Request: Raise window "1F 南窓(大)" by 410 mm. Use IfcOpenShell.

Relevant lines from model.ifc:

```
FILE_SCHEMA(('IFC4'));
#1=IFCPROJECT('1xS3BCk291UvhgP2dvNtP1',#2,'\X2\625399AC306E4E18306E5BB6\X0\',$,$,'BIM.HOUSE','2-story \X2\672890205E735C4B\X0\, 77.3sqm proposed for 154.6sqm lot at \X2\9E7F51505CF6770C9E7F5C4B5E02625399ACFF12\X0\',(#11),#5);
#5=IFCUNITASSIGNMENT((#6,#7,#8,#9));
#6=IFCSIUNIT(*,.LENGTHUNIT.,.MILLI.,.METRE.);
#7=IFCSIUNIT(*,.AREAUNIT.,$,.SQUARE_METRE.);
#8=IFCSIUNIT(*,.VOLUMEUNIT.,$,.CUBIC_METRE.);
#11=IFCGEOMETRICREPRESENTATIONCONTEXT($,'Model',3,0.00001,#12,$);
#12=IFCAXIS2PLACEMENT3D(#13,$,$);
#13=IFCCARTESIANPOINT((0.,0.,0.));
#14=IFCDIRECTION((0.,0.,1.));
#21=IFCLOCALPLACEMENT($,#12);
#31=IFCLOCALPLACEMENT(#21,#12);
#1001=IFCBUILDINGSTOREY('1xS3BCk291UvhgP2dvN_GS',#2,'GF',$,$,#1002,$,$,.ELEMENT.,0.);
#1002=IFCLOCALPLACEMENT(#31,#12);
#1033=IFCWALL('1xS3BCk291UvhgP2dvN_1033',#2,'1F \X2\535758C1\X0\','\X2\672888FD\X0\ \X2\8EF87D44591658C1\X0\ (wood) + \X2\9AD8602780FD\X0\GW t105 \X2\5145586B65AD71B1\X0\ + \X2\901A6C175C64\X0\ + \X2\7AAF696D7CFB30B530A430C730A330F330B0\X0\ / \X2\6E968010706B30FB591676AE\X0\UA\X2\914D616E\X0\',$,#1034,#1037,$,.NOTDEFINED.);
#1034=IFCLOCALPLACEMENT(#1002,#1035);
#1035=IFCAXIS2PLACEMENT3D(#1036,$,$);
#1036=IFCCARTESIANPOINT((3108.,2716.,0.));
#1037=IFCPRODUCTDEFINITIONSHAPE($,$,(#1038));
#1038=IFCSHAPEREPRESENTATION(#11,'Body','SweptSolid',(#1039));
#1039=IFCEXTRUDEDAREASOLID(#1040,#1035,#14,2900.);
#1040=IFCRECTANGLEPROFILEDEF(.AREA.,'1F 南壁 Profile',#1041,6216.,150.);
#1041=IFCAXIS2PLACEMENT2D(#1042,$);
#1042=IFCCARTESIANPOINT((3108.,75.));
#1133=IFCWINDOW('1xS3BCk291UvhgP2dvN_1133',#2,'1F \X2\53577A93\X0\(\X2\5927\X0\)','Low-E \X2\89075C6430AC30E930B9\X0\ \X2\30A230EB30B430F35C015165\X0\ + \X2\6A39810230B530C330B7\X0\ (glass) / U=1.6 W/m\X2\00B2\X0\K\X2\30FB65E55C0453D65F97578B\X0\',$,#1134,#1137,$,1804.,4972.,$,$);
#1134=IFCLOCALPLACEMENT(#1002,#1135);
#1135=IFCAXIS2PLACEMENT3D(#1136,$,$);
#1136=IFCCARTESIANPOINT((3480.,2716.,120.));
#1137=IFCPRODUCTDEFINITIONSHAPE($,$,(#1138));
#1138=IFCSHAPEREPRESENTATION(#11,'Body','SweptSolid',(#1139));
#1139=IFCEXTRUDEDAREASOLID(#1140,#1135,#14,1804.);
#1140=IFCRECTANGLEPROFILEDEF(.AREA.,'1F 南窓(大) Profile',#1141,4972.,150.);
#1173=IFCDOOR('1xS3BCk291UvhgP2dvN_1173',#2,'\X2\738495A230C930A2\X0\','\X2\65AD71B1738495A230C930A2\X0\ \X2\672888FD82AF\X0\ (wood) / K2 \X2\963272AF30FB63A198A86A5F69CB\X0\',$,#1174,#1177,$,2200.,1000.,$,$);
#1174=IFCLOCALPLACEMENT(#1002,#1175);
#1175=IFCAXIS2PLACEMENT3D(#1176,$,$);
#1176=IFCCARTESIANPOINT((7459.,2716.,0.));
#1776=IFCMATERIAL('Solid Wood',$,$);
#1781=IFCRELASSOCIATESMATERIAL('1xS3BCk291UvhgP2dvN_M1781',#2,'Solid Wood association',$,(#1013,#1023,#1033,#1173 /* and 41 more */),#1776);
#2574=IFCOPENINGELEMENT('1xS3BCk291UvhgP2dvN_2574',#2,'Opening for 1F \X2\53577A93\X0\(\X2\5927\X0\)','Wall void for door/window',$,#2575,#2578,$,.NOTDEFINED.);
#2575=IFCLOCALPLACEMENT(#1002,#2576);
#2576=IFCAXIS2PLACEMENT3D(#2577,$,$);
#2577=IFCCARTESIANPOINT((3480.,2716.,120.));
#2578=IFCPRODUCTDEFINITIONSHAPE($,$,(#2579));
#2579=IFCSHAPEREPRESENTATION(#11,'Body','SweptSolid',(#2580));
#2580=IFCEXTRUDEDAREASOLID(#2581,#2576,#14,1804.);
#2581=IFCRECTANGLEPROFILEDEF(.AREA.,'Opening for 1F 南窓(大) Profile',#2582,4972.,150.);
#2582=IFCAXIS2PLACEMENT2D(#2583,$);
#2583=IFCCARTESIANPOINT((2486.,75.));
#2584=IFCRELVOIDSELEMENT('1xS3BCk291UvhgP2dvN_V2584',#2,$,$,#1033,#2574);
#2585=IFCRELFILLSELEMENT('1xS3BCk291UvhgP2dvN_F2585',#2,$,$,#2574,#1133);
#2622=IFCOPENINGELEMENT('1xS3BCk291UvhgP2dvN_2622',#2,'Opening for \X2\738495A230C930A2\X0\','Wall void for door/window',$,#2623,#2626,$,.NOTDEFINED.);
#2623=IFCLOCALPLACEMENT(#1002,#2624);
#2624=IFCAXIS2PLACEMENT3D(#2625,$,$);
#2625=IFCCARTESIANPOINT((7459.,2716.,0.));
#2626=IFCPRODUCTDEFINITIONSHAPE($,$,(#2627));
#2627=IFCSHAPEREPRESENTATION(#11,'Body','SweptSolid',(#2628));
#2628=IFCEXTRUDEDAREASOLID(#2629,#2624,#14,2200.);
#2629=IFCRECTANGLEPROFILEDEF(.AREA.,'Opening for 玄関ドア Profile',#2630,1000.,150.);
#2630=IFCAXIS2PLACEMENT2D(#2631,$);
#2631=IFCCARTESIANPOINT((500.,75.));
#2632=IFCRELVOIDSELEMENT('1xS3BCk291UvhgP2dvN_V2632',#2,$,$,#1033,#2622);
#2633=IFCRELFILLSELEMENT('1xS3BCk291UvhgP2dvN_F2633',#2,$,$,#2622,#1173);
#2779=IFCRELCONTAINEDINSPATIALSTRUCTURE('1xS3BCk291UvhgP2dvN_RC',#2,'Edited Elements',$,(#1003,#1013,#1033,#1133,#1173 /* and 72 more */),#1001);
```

```python
import numpy as np
import ifcopenshell
import ifcopenshell.api.geometry
import ifcopenshell.util.placement
import ifcopenshell.util.unit

model = ifcopenshell.open("model.ifc")
unit_scale = ifcopenshell.util.unit.calculate_unit_scale(model)

window = model.by_id(1133)
opening = window.FillsVoids[0].RelatingOpeningElement
dz = 0.41 / unit_scale

shift = np.array([0.0, 0.0, dz])
# The window is not placed relative to its opening, so move both.
for product in (opening, window):
    matrix = ifcopenshell.util.placement.get_local_placement(product.ObjectPlacement)
    matrix[:3, 3] += shift
    ifcopenshell.api.geometry.edit_object_placement(model, product=product, matrix=matrix, is_si=False)

print(f"moved by {dz * unit_scale:+.3f} m")

model.write("model-out.ifc")
```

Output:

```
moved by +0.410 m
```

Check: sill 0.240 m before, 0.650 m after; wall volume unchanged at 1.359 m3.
